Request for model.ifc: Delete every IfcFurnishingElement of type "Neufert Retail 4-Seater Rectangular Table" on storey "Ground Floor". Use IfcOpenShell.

First a look at what the model holds.

```python
import ifcopenshell
import ifcopenshell.util.element

model = ifcopenshell.open("model.ifc")
print(model.schema)
storey = next(s for s in model.by_type("IfcBuildingStorey") if s.Name == "Ground Floor")
furniture = [e for e in ifcopenshell.util.element.get_decomposition(storey) if e.is_a("IfcFurnishingElement")]
seen = {}
for e in furniture:
    element_type = ifcopenshell.util.element.get_type(e)
    name = element_type.Name if element_type not in (None, e) else None
    seen[name] = seen.get(name, 0) + 1
for name, count in sorted(seen.items(), key=str):
    print(count, "x", name)
```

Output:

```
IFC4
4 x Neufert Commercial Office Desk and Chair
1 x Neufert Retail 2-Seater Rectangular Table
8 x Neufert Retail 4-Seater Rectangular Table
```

```python
import ifcopenshell
import ifcopenshell.api.root
import ifcopenshell.util.element

model = ifcopenshell.open("model.ifc")

storey = next(s for s in model.by_type("IfcBuildingStorey") if s.Name == "Ground Floor")
furniture = [e for e in ifcopenshell.util.element.get_decomposition(storey) if e.is_a("IfcFurnishingElement")]
targets = [e for e in furniture if (t := ifcopenshell.util.element.get_type(e)) not in (None, e) and t.Name == "Neufert Retail 4-Seater Rectangular Table"]

for e in targets:
    ifcopenshell.api.root.remove_product(model, product=e)
print(len(targets), "removed")

model.write("model_v2.ifc")
```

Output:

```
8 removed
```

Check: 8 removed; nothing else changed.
